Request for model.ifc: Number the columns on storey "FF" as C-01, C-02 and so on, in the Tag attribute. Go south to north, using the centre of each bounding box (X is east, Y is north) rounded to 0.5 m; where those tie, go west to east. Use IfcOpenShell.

First a look at what the model holds.

```python
import ifcopenshell
import ifcopenshell.util.element
import ifcopenshell.util.placement

model = ifcopenshell.open("model.ifc")
print(model.schema)
storey = next(s for s in model.by_type("IfcBuildingStorey") if s.Name == "FF")
columns = [e for e in ifcopenshell.util.element.get_decomposition(storey) if e.is_a("IfcColumn")]
for e in sorted(columns, key=lambda e: e.id()):
    origin = ifcopenshell.util.placement.get_local_placement(e.ObjectPlacement)[:3, 3]
    print(e.id(), e.Tag, e.Name, origin.round(2) + 0.0, sep=" | ")
```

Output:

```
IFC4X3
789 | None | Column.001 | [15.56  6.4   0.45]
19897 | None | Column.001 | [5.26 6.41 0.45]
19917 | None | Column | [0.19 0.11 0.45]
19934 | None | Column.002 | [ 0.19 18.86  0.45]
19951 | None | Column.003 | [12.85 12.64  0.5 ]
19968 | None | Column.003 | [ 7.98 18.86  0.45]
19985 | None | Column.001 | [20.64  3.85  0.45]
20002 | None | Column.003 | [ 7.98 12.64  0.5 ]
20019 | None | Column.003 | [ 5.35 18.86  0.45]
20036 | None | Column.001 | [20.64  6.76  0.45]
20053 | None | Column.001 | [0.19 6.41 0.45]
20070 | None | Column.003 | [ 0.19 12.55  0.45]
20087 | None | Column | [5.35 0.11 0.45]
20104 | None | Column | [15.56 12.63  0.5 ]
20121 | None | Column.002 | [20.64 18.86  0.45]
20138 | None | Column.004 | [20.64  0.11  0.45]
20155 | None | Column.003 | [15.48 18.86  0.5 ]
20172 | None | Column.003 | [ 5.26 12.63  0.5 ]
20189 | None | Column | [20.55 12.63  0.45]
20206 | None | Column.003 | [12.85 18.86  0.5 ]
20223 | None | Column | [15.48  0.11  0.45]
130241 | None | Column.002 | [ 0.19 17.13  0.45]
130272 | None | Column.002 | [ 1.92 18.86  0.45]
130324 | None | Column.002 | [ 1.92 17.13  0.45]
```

```python
import ifcopenshell
import ifcopenshell.geom
import ifcopenshell.util.element
import ifcopenshell.util.shape

model = ifcopenshell.open("model.ifc")
settings = ifcopenshell.geom.settings()
settings.set("use-world-coords", True)


def centre(element):
    shape = ifcopenshell.geom.create_shape(settings, element)
    return ifcopenshell.util.shape.get_bbox_centroid(shape.geometry)


storey = next(s for s in model.by_type("IfcBuildingStorey") if s.Name == "FF")
columns = [e for e in ifcopenshell.util.element.get_decomposition(storey) if e.is_a("IfcColumn")]

# Insertion points can sit at a corner or the storey origin, so sort by the geometry (in metres).
centres = {e: centre(e) for e in columns}
columns.sort(key=lambda e: (round(centres[e][1] / 0.5), centres[e][0]))

for i, e in enumerate(columns, start=1):
    number = f"C-{i:02d}"
    e.Tag = number
    print(e.id(), number)

model.write("model_rev.ifc")
```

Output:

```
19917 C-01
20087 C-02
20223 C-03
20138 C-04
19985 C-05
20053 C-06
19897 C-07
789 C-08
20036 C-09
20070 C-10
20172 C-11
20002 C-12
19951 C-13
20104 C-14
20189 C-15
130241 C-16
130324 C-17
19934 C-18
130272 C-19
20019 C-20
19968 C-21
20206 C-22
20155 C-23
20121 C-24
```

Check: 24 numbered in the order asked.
